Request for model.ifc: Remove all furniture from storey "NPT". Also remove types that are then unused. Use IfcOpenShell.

First a look at what the model holds.

```python
import ifcopenshell
import ifcopenshell.util.element

model = ifcopenshell.open("model.ifc")
print(model.schema)
storey = next(s for s in model.by_type("IfcBuildingStorey") if s.Name == "NPT")
furniture = [e for e in ifcopenshell.util.element.get_decomposition(storey) if e.is_a("IfcFurnishingElement")]
seen = {}
for e in furniture:
    element_type = ifcopenshell.util.element.get_type(e)
    name = element_type.Name if element_type not in (None, e) else None
    seen[name] = seen.get(name, 0) + 1
for name, count in sorted(seen.items(), key=str):
    print(count, "x", name)
```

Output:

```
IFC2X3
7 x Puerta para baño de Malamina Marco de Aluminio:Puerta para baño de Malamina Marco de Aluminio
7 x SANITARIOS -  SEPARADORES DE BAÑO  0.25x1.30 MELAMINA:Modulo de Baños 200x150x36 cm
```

```python
import ifcopenshell
import ifcopenshell.api.root
import ifcopenshell.util.element

model = ifcopenshell.open("model.ifc")

storey = next(s for s in model.by_type("IfcBuildingStorey") if s.Name == "NPT")
furniture = [e for e in ifcopenshell.util.element.get_decomposition(storey) if e.is_a("IfcFurnishingElement")]
types = {ifcopenshell.util.element.get_type(e) for e in furniture} - {None, *furniture}

for e in furniture:
    ifcopenshell.api.root.remove_product(model, product=e)
print(len(furniture), "removed")

unused = [t for t in types if not ifcopenshell.util.element.get_types(t)]
for t in unused:
    ifcopenshell.api.root.remove_product(model, product=t)
print(len(unused), "unused types removed")

model.write("model_updated.ifc")
```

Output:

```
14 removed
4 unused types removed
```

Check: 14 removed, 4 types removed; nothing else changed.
